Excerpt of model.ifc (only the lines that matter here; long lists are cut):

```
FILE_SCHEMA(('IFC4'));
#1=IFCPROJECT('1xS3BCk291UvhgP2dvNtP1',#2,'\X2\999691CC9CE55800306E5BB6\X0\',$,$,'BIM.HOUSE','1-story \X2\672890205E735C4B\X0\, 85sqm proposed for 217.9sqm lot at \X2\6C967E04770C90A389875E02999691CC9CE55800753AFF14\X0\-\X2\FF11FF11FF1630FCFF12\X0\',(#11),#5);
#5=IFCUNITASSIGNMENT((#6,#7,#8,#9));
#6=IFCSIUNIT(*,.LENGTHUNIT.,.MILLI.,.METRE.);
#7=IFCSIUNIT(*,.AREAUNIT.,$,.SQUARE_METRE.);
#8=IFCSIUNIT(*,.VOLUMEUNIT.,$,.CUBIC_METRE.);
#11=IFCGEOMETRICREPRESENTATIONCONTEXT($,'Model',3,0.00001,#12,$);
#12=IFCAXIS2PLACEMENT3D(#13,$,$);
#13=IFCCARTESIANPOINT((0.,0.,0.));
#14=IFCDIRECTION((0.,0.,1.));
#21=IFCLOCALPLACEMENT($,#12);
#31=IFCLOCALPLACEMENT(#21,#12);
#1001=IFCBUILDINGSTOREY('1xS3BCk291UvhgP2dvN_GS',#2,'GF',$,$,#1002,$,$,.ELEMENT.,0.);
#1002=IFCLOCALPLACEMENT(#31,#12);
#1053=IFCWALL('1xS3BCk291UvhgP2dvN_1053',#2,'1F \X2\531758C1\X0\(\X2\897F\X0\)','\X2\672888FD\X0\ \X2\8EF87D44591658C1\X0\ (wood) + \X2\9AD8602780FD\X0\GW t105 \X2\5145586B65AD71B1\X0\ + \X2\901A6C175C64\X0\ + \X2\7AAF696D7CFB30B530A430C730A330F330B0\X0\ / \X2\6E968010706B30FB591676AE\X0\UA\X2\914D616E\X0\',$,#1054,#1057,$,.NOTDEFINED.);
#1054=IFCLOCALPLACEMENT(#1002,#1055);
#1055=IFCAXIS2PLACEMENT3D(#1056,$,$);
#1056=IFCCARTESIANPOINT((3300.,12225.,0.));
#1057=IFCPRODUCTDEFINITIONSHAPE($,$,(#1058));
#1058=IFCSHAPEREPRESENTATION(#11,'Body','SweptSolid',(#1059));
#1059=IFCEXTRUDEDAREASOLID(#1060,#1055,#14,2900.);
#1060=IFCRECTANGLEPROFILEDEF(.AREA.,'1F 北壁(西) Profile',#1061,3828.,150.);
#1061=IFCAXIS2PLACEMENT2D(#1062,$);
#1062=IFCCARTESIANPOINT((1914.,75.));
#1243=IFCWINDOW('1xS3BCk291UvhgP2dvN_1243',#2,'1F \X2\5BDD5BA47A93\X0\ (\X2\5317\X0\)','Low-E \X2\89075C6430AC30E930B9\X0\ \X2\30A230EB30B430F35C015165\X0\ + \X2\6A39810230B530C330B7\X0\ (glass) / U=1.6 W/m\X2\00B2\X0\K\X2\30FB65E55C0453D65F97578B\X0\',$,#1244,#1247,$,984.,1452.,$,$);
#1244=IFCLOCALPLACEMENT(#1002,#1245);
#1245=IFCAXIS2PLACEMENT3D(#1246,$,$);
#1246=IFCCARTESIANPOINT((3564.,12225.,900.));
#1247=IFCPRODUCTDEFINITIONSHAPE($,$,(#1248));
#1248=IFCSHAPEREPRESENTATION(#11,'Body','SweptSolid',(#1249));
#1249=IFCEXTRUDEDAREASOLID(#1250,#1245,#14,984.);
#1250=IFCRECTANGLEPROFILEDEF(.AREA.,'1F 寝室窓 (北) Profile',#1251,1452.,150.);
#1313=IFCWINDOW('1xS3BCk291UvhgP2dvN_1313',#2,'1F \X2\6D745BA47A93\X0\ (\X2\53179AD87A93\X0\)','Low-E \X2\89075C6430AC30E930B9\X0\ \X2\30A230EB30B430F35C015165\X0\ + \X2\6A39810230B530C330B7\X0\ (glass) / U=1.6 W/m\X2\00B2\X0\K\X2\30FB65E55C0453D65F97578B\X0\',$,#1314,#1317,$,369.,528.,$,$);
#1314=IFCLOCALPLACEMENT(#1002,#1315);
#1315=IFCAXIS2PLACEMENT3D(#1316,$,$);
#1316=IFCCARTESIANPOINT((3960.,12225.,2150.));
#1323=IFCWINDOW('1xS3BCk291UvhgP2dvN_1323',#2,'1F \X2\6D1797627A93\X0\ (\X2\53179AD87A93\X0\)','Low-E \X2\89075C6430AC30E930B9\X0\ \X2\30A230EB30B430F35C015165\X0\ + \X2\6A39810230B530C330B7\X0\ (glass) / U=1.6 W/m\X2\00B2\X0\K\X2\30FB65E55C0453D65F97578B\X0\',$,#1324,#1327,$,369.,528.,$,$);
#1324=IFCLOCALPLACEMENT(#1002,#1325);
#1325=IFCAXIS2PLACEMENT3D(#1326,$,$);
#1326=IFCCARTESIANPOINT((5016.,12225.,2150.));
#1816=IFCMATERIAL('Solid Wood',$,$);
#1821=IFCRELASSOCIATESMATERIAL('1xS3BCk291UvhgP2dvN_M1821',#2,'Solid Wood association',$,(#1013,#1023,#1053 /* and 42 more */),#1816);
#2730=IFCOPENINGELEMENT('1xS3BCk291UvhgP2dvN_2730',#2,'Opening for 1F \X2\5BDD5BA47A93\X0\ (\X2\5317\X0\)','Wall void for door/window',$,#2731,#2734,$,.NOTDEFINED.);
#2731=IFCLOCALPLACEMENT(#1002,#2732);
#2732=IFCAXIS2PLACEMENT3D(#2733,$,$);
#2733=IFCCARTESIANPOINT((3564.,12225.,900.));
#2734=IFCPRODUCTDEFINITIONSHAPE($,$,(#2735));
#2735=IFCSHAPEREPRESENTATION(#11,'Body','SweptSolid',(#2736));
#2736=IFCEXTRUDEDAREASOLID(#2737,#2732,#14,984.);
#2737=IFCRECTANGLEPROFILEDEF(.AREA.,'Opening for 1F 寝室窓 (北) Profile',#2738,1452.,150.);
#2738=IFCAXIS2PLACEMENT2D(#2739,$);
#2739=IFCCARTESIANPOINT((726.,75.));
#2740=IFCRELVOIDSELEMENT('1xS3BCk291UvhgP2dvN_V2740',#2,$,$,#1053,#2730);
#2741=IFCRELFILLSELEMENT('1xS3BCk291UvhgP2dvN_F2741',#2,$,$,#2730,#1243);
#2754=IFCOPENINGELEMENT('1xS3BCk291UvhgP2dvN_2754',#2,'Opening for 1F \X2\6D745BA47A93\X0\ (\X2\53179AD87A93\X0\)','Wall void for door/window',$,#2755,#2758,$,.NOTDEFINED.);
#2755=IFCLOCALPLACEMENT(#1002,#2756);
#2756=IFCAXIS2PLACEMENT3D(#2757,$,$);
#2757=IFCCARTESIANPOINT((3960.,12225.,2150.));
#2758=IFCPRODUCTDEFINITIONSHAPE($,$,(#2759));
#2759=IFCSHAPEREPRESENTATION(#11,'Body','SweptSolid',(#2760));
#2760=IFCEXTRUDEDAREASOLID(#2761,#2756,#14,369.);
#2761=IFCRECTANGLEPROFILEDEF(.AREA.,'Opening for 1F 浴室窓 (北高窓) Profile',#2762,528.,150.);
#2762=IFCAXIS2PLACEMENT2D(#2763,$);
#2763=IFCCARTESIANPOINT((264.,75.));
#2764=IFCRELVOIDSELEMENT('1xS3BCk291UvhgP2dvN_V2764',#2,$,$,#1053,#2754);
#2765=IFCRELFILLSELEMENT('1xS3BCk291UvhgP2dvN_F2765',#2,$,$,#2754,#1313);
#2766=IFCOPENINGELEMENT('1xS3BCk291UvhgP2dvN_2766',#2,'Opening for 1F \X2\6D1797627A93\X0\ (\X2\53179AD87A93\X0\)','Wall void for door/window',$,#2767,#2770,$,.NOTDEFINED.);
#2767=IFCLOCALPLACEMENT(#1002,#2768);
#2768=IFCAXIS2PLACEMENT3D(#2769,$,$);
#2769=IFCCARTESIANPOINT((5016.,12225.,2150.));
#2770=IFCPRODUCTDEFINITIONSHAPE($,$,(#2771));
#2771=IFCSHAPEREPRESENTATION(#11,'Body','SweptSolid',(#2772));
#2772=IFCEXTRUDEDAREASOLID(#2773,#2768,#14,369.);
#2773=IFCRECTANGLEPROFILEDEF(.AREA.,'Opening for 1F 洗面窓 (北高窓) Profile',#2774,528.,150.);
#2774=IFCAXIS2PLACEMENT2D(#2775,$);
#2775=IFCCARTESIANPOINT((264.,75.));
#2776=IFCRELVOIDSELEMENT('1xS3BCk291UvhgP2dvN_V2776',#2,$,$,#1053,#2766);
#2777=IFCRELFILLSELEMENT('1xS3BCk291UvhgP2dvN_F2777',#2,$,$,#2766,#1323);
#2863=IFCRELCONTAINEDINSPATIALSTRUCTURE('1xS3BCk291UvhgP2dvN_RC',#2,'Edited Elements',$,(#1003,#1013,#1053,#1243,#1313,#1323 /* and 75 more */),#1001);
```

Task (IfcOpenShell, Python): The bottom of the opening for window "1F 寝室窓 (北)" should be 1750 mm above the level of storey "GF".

```python
import numpy as np
import ifcopenshell
import ifcopenshell.api.geometry
import ifcopenshell.geom
import ifcopenshell.util.element
import ifcopenshell.util.placement
import ifcopenshell.util.shape
import ifcopenshell.util.unit

model = ifcopenshell.open("model.ifc")
unit_scale = ifcopenshell.util.unit.calculate_unit_scale(model)

window = model.by_guid("1xS3BCk291UvhgP2dvN_1243")
opening = window.FillsVoids[0].RelatingOpeningElement
storey = ifcopenshell.util.element.get_container(window, ifc_class="IfcBuildingStorey")
level = ifcopenshell.util.placement.get_local_placement(storey.ObjectPlacement)[2, 3]

# The opening's origin need not be at the sill, so measure its lowest point.
shape = ifcopenshell.geom.create_shape(ifcopenshell.geom.settings(), opening)
bottom = ifcopenshell.util.shape.get_shape_bottom_elevation(shape, shape.geometry) / unit_scale
dz = level + 1.75 / unit_scale - bottom

shift = np.array([0.0, 0.0, dz])
# The window is not placed relative to its opening, so move both.
for product in (opening, window):
    matrix = ifcopenshell.util.placement.get_local_placement(product.ObjectPlacement)
    matrix[:3, 3] += shift
    ifcopenshell.api.geometry.edit_object_placement(model, product=product, matrix=matrix, is_si=False)

print(f"moved by {dz * unit_scale:+.3f} m")

model.write("model_updated.ifc")
```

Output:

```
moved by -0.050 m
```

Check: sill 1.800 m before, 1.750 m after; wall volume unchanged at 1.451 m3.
